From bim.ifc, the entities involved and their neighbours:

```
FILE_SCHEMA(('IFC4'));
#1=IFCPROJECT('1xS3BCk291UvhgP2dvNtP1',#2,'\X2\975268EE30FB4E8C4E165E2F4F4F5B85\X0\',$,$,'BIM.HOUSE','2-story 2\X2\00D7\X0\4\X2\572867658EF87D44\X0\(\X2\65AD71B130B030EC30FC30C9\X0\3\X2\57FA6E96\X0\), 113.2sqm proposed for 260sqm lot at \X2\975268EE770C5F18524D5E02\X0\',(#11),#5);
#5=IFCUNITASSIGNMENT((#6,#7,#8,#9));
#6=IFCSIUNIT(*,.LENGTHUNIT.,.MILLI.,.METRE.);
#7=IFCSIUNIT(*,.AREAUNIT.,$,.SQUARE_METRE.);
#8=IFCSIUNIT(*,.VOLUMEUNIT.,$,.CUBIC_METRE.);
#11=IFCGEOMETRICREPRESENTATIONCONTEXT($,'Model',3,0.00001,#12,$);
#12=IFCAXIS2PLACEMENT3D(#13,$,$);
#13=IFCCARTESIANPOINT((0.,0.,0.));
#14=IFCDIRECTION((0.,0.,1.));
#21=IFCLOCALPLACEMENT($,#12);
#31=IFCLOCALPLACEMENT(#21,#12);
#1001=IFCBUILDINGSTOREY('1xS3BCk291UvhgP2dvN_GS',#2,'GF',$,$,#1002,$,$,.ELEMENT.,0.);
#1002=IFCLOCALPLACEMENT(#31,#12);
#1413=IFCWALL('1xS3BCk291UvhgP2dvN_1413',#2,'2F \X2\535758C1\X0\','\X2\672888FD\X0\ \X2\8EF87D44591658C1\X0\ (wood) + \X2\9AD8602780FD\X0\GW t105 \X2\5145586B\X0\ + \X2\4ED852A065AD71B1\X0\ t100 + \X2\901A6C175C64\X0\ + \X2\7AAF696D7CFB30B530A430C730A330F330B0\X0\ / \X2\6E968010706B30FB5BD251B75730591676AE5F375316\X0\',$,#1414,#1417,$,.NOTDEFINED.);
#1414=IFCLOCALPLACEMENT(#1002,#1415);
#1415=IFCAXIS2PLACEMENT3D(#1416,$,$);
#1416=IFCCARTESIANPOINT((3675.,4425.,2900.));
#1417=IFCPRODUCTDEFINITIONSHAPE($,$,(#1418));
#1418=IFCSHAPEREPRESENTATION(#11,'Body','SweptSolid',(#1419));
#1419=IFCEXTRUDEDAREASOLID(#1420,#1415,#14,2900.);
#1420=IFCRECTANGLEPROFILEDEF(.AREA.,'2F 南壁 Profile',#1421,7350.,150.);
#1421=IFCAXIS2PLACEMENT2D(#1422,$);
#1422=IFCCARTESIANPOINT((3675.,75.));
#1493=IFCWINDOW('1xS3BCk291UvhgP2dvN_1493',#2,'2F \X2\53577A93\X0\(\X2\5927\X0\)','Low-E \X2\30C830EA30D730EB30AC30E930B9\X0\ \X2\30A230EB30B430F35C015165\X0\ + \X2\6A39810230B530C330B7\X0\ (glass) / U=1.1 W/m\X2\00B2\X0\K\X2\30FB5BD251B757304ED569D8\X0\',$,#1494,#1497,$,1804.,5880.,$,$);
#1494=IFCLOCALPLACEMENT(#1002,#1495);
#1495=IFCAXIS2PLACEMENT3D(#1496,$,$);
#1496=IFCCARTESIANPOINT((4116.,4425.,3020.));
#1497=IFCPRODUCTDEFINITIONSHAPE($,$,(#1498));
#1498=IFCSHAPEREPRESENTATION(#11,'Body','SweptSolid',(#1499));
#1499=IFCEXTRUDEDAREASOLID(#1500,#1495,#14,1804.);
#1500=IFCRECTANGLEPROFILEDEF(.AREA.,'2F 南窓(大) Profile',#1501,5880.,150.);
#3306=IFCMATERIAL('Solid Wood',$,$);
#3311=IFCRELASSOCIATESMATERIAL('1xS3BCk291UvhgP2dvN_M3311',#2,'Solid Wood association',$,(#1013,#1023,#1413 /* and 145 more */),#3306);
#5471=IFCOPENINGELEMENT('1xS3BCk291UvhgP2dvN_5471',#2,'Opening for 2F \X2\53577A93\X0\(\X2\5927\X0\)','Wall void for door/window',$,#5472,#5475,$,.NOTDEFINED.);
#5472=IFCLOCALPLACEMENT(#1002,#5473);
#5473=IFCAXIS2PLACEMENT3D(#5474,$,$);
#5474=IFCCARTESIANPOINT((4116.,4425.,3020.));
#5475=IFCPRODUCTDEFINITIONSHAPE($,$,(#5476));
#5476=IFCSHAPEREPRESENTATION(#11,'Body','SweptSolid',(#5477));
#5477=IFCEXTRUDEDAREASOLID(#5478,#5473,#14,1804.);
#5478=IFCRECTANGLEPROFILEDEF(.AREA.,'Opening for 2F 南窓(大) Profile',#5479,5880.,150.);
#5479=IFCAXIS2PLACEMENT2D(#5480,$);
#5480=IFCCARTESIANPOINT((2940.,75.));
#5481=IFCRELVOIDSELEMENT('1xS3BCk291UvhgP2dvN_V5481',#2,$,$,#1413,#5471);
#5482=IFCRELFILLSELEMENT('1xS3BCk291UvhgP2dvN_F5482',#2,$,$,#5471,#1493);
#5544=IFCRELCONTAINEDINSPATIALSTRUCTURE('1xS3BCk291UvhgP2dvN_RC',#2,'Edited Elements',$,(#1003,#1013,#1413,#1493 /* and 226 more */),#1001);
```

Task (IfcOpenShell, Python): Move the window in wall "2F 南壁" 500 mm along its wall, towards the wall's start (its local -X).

```python
import ifcopenshell
import ifcopenshell.api.geometry
import ifcopenshell.util.placement
import ifcopenshell.util.unit

model = ifcopenshell.open("bim.ifc")
unit_scale = ifcopenshell.util.unit.calculate_unit_scale(model)

window = model.by_guid("1xS3BCk291UvhgP2dvN_1493")
opening = window.FillsVoids[0].RelatingOpeningElement
wall = opening.VoidsElements[0].RelatingBuildingElement

wall_matrix = ifcopenshell.util.placement.get_local_placement(wall.ObjectPlacement)
shift = wall_matrix[:3, 0] * -0.5 / unit_scale
before = ifcopenshell.util.placement.get_local_placement(window.ObjectPlacement)[:3, 3].copy()

# The window is not placed relative to its opening, so move both.
for product in (opening, window):
    matrix = ifcopenshell.util.placement.get_local_placement(product.ObjectPlacement)
    matrix[:3, 3] += shift
    ifcopenshell.api.geometry.edit_object_placement(model, product=product, matrix=matrix, is_si=False)

after = ifcopenshell.util.placement.get_local_placement(window.ObjectPlacement)[:3, 3]
print("window moved by", (after - before).round(3) + 0.0)

model.write("bim_updated.ifc")
```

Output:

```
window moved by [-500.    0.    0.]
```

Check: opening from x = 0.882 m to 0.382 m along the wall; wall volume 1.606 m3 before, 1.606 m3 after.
